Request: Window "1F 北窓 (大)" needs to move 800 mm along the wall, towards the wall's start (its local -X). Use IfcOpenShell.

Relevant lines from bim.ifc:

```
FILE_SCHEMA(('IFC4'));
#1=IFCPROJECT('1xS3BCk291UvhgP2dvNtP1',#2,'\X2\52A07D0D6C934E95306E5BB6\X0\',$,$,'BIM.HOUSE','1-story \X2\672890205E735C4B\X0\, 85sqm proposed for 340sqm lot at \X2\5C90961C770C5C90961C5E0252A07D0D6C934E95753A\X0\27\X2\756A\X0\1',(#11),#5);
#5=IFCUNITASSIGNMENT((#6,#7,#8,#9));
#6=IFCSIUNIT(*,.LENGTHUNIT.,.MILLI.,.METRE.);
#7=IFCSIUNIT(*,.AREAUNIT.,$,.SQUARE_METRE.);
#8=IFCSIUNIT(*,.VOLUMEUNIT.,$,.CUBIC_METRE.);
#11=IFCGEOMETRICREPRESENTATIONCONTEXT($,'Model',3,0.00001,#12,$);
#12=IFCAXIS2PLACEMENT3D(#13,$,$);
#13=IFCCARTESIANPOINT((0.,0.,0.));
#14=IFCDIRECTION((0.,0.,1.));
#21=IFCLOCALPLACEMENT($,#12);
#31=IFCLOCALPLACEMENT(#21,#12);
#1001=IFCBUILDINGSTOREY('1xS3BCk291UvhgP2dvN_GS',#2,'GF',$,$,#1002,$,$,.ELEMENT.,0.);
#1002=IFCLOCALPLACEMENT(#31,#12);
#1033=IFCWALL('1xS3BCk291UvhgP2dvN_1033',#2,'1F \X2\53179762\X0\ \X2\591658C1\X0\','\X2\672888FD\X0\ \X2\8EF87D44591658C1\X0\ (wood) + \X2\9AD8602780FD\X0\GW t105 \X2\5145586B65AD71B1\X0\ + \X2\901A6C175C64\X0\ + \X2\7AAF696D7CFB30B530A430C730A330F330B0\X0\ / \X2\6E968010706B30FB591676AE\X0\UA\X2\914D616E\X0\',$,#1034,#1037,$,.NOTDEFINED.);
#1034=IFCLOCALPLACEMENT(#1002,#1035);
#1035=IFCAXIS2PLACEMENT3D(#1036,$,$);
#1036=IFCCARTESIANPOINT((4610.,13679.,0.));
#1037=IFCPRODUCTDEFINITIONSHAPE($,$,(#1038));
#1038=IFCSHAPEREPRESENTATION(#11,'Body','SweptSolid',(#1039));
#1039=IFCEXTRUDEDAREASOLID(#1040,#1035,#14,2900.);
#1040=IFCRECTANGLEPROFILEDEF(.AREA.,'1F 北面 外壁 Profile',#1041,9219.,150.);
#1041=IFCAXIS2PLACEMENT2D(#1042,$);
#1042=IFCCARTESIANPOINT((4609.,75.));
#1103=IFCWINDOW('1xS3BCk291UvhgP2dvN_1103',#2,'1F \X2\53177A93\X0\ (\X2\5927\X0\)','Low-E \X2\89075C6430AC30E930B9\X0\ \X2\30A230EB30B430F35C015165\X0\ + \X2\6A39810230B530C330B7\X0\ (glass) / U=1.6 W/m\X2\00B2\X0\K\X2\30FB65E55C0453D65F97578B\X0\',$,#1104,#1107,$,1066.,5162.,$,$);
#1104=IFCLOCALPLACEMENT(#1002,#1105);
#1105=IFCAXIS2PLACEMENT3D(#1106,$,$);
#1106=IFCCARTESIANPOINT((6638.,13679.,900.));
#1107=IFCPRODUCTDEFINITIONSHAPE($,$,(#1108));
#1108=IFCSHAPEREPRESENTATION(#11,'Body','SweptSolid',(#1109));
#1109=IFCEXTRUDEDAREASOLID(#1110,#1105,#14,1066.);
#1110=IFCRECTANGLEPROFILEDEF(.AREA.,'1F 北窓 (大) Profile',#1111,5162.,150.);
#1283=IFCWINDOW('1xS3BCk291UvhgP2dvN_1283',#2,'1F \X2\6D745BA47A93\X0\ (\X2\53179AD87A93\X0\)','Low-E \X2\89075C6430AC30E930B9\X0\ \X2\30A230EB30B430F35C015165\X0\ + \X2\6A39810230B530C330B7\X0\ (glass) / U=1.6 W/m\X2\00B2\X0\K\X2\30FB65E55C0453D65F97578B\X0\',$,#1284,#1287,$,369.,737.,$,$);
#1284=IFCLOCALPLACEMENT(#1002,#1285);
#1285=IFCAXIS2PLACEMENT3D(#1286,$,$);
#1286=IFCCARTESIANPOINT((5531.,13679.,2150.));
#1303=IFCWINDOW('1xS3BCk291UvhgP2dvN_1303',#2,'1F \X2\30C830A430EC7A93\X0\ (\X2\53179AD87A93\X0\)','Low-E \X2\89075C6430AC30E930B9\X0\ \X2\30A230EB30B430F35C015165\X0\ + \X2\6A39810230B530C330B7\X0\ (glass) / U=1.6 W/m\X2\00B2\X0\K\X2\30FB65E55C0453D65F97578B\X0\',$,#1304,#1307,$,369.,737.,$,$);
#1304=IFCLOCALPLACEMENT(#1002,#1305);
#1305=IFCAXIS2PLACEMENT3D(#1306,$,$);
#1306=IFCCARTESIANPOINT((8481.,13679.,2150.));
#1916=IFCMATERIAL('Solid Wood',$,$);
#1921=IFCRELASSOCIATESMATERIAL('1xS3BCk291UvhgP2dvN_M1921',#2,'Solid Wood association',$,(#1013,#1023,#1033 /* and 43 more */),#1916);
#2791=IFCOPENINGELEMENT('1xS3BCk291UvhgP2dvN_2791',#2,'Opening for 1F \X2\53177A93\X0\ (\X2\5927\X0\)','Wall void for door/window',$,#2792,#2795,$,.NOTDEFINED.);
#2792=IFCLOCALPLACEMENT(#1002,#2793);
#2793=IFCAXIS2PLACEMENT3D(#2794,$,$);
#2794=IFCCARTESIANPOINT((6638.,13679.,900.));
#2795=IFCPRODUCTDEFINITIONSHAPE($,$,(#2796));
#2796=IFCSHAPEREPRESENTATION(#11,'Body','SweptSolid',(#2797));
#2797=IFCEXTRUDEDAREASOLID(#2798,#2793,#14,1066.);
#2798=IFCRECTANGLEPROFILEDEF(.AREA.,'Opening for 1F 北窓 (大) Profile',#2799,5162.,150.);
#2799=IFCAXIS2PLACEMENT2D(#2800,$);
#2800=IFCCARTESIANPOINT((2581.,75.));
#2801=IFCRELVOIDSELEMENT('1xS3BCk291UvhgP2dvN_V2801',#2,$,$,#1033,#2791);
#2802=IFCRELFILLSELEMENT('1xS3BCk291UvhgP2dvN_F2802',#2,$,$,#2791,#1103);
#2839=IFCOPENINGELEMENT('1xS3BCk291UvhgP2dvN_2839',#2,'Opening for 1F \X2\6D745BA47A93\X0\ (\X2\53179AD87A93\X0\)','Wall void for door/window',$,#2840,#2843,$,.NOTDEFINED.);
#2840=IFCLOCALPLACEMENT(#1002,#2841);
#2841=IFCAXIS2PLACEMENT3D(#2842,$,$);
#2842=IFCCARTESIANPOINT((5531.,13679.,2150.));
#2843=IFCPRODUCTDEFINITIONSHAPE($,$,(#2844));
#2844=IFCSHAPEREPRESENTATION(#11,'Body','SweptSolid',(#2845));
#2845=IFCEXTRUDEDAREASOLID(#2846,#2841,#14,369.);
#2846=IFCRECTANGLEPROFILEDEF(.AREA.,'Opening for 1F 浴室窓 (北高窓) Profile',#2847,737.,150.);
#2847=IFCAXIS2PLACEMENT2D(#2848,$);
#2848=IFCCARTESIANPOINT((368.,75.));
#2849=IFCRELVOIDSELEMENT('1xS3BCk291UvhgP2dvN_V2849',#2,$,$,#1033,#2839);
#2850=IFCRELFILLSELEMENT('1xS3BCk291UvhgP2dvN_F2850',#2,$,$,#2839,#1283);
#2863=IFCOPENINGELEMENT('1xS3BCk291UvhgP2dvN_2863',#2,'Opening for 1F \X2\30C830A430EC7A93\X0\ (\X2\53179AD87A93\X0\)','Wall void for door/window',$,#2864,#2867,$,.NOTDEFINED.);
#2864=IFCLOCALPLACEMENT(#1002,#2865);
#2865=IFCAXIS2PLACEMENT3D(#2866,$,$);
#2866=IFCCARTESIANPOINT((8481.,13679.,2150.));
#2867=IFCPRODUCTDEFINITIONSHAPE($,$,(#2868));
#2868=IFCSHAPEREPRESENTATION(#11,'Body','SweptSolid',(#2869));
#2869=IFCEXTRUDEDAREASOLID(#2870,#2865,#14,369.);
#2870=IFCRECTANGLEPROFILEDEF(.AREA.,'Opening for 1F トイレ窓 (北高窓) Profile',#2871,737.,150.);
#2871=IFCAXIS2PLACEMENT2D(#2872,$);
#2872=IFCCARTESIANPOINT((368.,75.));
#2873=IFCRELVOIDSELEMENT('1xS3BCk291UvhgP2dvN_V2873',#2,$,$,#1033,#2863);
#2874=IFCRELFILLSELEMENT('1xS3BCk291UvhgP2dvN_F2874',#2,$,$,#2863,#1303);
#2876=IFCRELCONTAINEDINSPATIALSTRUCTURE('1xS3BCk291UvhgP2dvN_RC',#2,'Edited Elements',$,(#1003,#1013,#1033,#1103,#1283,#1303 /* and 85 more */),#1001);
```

```python
import ifcopenshell
import ifcopenshell.api.geometry
import ifcopenshell.util.placement

model = ifcopenshell.open("bim.ifc")

window = model.by_guid("1xS3BCk291UvhgP2dvN_1103")
opening = window.FillsVoids[0].RelatingOpeningElement
wall = opening.VoidsElements[0].RelatingBuildingElement

wall_matrix = ifcopenshell.util.placement.get_local_placement(wall.ObjectPlacement)
shift = wall_matrix[:3, 0] * -800.0
before = ifcopenshell.util.placement.get_local_placement(window.ObjectPlacement)[:3, 3].copy()

# The window is not placed relative to its opening, so move both.
for product in (opening, window):
    matrix = ifcopenshell.util.placement.get_local_placement(product.ObjectPlacement)
    matrix[:3, 3] += shift
    ifcopenshell.api.geometry.edit_object_placement(model, product=product, matrix=matrix, is_si=False)

after = ifcopenshell.util.placement.get_local_placement(window.ObjectPlacement)[:3, 3]
print("window moved by", (after - before).round(3) + 0.0)

model.write("bim_rev.ifc")
```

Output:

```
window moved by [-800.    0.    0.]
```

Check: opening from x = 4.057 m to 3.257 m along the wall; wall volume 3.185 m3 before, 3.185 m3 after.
